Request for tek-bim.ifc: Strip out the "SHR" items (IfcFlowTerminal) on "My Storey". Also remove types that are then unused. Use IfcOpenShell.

First a look at what the model holds.

```python
import ifcopenshell
import ifcopenshell.util.element

model = ifcopenshell.open("tek-bim.ifc")
print(model.schema)
storey = next(s for s in model.by_type("IfcBuildingStorey") if s.Name == "My Storey")
terminals = [e for e in ifcopenshell.util.element.get_decomposition(storey) if e.is_a("IfcFlowTerminal")]
seen = {}
for e in terminals:
    element_type = ifcopenshell.util.element.get_type(e)
    name = element_type.Name if element_type not in (None, e) else None
    seen[name] = seen.get(name, 0) + 1
for name, count in sorted(seen.items(), key=str):
    print(count, "x", name)
```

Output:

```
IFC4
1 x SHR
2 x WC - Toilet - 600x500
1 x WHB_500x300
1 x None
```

```python
import ifcopenshell
import ifcopenshell.api.root
import ifcopenshell.util.element

model = ifcopenshell.open("tek-bim.ifc")

storey = next(s for s in model.by_type("IfcBuildingStorey") if s.Name == "My Storey")
terminals = [e for e in ifcopenshell.util.element.get_decomposition(storey) if e.is_a("IfcFlowTerminal")]
targets = [e for e in terminals if (t := ifcopenshell.util.element.get_type(e)) not in (None, e) and t.Name == "SHR"]
types = {ifcopenshell.util.element.get_type(e) for e in targets} - {None, *targets}

for e in targets:
    ifcopenshell.api.root.remove_product(model, product=e)
print(len(targets), "removed")

unused = [t for t in types if not ifcopenshell.util.element.get_types(t)]
for t in unused:
    ifcopenshell.api.root.remove_product(model, product=t)
print(len(unused), "unused types removed")

model.write("tek-bim_edited.ifc")
```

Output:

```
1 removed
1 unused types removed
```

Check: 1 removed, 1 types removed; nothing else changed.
